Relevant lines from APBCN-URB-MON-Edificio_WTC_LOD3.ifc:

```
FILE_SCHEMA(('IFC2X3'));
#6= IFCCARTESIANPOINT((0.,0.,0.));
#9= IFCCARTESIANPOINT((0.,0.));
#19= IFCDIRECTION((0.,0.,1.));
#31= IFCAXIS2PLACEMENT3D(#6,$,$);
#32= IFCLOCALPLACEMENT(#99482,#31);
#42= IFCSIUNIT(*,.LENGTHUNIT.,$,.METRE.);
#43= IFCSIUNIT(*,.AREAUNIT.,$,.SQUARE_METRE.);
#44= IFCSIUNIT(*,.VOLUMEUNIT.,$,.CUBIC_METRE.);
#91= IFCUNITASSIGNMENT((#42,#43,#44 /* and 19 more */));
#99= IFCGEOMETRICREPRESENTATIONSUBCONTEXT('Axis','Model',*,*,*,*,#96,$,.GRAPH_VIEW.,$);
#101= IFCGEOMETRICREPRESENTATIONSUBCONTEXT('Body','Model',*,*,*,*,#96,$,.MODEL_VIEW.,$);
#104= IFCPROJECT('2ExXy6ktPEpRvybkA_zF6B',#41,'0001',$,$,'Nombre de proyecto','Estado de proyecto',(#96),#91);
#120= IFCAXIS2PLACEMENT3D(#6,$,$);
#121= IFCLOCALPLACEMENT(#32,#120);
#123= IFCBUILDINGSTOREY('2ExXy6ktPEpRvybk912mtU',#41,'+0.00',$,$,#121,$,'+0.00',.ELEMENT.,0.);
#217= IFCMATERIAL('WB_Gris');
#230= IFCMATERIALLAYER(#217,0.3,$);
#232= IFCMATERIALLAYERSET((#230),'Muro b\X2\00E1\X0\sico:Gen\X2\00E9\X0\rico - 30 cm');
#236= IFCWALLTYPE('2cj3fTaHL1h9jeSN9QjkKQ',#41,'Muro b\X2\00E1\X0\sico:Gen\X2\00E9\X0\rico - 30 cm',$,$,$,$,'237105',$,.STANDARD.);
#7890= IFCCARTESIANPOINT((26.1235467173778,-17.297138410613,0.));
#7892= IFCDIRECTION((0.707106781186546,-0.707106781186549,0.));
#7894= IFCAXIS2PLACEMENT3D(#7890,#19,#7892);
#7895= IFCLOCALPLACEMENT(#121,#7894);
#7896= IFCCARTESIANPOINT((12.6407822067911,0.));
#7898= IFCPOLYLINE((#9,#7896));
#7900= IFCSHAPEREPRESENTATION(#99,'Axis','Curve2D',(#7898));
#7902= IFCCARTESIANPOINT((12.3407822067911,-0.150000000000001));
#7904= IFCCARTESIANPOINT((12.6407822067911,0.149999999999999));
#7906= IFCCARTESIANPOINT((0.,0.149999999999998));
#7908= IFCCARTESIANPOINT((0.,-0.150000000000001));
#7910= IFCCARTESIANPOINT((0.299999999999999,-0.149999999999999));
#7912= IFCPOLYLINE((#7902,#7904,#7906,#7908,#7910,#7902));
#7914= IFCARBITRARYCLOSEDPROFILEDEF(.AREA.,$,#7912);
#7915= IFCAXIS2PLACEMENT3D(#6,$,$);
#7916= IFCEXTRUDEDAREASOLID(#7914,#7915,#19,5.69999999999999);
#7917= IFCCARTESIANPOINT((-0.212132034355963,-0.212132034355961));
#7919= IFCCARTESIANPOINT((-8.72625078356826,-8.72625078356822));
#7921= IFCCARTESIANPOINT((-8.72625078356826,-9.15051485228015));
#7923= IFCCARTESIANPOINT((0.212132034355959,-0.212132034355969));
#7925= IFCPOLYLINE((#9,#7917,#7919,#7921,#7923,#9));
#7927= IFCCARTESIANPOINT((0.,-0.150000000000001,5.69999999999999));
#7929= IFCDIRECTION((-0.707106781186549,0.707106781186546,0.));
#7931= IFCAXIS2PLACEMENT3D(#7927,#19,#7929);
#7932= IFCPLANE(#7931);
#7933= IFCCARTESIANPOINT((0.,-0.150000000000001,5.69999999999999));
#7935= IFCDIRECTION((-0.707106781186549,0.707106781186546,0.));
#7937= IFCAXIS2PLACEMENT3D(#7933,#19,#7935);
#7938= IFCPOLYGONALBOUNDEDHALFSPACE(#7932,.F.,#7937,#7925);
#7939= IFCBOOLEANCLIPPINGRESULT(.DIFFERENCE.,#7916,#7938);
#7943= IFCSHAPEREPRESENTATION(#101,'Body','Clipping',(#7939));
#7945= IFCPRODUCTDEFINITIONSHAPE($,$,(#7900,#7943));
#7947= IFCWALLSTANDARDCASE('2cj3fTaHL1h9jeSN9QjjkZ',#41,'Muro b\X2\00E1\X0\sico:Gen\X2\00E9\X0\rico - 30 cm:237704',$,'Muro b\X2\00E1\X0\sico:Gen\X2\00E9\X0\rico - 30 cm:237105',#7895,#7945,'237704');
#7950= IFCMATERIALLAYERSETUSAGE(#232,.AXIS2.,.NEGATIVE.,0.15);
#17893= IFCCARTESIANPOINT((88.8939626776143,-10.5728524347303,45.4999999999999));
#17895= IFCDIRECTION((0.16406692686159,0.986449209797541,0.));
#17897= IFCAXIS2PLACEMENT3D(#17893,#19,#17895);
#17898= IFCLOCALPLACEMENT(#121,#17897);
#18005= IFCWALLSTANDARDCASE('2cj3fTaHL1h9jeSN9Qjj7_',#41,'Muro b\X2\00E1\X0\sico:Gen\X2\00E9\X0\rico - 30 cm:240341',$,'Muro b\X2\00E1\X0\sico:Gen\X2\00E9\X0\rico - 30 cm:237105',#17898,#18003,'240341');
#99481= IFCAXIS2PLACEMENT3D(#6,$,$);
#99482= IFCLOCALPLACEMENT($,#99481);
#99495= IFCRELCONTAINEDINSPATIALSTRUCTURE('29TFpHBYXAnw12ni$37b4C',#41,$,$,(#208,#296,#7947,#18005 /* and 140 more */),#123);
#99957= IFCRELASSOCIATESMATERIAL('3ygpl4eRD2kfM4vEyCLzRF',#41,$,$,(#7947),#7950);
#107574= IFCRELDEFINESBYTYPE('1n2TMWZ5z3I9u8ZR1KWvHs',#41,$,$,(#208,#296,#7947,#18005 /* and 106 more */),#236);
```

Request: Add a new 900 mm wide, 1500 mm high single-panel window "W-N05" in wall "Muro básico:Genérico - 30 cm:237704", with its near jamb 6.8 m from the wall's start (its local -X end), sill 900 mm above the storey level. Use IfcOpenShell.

```python
import numpy as np
import ifcopenshell
import ifcopenshell.api.feature
import ifcopenshell.api.geometry
import ifcopenshell.api.root
import ifcopenshell.api.spatial
import ifcopenshell.api.type
import ifcopenshell.geom
import ifcopenshell.util.element
import ifcopenshell.util.placement
import ifcopenshell.util.representation
import ifcopenshell.util.shape
import ifcopenshell.util.unit

model = ifcopenshell.open("APBCN-URB-MON-Edificio_WTC_LOD3.ifc")
unit_scale = ifcopenshell.util.unit.calculate_unit_scale(model)
settings = ifcopenshell.geom.settings()


def volume(element):
    """Net volume in cubic metres, openings subtracted."""
    shape = ifcopenshell.geom.create_shape(settings, element)
    return ifcopenshell.util.shape.get_volume(shape.geometry)


wall = model.by_id(7947)
storey = ifcopenshell.util.element.get_container(wall, ifc_class="IfcBuildingStorey")
context = ifcopenshell.util.representation.get_context(model, "Model", "Body", "MODEL_VIEW")
before = volume(wall)

width, height, from_end, sill = 0.9, 1.5, 6.8, 0.9  # metres

# The wall runs along its own X axis, and the end named is its -X end.
wall_shape = ifcopenshell.geom.create_shape(settings, wall)
x, y, z = ifcopenshell.util.shape.get_vertices(wall_shape.geometry).T
start = x.min() + from_end
face, thickness = float(y.min()), float(y.max() - y.min())
wall_matrix = ifcopenshell.util.placement.get_local_placement(wall.ObjectPlacement)
level = ifcopenshell.util.placement.get_local_placement(storey.ObjectPlacement)[2, 3]


def in_wall(x, y):
    """Placement at x, y metres in the wall's axes, at sill height."""
    matrix = wall_matrix.copy()
    matrix[:, 3] = wall_matrix @ np.array([x / unit_scale, y / unit_scale, 0.0, 1.0])
    matrix[2, 3] = level + sill / unit_scale
    return matrix


# Opening: a box that overshoots both wall faces by 50 mm.
opening = ifcopenshell.api.root.create_entity(model, ifc_class="IfcOpeningElement")
box = ifcopenshell.api.geometry.add_wall_representation(
    model, context=context, length=width, height=height, thickness=thickness + 0.1
)
ifcopenshell.api.geometry.assign_representation(model, product=opening, representation=box)
ifcopenshell.api.geometry.edit_object_placement(model, product=opening, matrix=in_wall(start, face - 0.05), is_si=False)
ifcopenshell.api.feature.add_feature(model, feature=opening, element=wall)

window = ifcopenshell.api.root.create_entity(model, ifc_class="IfcWindow", name="W-N05")
window.OverallWidth, window.OverallHeight = width / unit_scale, height / unit_scale
body = ifcopenshell.api.geometry.add_window_representation(
    model,
    context=context,
    overall_width=window.OverallWidth,
    overall_height=window.OverallHeight,
    partition_type="SINGLE_PANEL",
)
ifcopenshell.api.geometry.assign_representation(model, product=window, representation=body)
ifcopenshell.api.spatial.assign_container(model, products=[window], relating_structure=storey)
fills = ifcopenshell.api.feature.add_filling(model, opening=opening, element=window)
fills.OwnerHistory = window.OwnerHistory  # required in IFC2X3

# IFC2X3 keeps the operation on the window style.
style = ifcopenshell.api.root.create_entity(model, ifc_class="IfcWindowStyle", name="W-N05")
style.OperationType, style.ConstructionType = "SINGLE_PANEL", "NOTDEFINED"
style.ParameterTakesPrecedence = style.Sizeable = False
ifcopenshell.api.type.assign_type(model, related_objects=[window], relating_type=style)

# Centre the window in the wall's thickness.
ifcopenshell.api.geometry.edit_object_placement(model, product=window, matrix=in_wall(start, face), is_si=False)
window_shape = ifcopenshell.geom.create_shape(settings, window)
depth = ifcopenshell.util.shape.get_vertices(window_shape.geometry)[:, 1]
offset = face + thickness / 2 - (depth.min() + depth.max()) / 2
ifcopenshell.api.geometry.edit_object_placement(model, product=window, matrix=in_wall(start, offset), is_si=False)

after = volume(wall)

print(f"wall volume {before:.3f} -> {after:.3f} m3")

model.write("APBCN-URB-MON-Edificio_WTC_LOD3_rev.ifc")
```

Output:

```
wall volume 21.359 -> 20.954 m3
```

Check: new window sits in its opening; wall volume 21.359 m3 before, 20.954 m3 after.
